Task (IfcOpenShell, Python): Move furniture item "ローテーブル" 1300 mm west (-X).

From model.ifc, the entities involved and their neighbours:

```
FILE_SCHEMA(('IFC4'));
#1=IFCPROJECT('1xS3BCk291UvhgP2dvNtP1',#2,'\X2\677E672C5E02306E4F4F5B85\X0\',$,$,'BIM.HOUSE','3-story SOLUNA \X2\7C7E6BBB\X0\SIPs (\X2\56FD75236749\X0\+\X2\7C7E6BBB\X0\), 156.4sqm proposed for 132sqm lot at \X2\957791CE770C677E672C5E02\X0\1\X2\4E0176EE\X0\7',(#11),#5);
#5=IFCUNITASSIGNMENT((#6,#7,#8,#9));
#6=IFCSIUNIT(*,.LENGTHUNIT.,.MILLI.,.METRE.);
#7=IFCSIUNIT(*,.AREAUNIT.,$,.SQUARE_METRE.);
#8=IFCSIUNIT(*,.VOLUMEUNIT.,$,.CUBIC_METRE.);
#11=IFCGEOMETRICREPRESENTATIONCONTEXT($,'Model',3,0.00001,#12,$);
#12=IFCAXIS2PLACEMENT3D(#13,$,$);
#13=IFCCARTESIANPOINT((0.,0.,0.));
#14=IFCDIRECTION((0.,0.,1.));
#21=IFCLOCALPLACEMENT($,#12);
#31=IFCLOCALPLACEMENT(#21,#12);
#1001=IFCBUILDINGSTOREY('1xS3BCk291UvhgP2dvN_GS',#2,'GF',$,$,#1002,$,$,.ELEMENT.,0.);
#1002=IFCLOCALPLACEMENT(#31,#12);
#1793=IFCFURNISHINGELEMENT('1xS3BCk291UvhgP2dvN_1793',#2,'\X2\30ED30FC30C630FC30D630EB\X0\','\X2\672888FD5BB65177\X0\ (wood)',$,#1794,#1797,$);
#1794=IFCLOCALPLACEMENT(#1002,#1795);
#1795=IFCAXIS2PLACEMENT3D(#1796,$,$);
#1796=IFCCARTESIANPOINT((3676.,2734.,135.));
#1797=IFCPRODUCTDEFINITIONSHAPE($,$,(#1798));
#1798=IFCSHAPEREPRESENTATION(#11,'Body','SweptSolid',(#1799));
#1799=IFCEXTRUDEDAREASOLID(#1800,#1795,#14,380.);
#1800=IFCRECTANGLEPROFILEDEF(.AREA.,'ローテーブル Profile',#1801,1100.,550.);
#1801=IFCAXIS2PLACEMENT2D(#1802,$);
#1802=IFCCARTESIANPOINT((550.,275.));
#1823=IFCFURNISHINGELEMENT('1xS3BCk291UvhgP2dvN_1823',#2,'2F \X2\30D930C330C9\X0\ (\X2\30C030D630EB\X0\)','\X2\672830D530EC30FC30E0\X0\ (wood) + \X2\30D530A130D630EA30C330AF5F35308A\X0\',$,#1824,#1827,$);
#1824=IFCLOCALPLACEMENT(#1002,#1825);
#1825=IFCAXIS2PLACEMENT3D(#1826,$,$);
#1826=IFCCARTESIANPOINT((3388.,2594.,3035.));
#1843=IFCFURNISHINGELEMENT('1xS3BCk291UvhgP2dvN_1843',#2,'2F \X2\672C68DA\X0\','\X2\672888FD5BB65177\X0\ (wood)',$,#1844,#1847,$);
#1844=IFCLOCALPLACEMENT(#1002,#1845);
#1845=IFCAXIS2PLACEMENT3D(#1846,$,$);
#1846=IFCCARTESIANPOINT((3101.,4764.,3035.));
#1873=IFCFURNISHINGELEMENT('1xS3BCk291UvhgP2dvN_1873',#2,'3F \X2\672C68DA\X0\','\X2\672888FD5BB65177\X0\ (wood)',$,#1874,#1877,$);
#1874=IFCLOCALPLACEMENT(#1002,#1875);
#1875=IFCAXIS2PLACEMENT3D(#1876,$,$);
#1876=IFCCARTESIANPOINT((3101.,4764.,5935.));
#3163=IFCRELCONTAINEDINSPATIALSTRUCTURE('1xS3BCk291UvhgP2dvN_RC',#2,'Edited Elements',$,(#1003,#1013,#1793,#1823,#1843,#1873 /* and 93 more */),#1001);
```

```python
import ifcopenshell
import ifcopenshell.api.geometry
import ifcopenshell.util.placement
import ifcopenshell.util.unit

model = ifcopenshell.open("model.ifc")
unit_scale = ifcopenshell.util.unit.calculate_unit_scale(model)

item = model.by_guid("1xS3BCk291UvhgP2dvN_1793")
matrix = ifcopenshell.util.placement.get_local_placement(item.ObjectPlacement)
matrix[0, 3] -= 1.3 / unit_scale
ifcopenshell.api.geometry.edit_object_placement(model, product=item, matrix=matrix, is_si=False)

print(ifcopenshell.util.placement.get_local_placement(item.ObjectPlacement).round(3) + 0.0)

model.write("model-out.ifc")
```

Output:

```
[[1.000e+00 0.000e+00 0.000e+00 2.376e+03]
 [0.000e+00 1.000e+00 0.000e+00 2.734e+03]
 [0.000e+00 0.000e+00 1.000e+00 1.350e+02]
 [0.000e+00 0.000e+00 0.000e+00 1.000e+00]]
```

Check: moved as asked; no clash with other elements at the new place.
